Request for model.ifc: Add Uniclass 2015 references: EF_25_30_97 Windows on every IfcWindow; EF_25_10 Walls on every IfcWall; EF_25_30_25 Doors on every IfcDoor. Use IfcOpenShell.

First a look at what the model holds.

```python
import ifcopenshell

model = ifcopenshell.open("model.ifc")
print(model.schema)
print("classifications:", [c.Name for c in model.by_type("IfcClassification")])
for ifc_class in ("IfcDoor", "IfcRoof", "IfcStair", "IfcWall", "IfcWindow"):
    print(ifc_class, len(model.by_type(ifc_class)))
```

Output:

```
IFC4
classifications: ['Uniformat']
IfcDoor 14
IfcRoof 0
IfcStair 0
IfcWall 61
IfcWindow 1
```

```python
import ifcopenshell
import ifcopenshell.api.classification

model = ifcopenshell.open("model.ifc")

system = ifcopenshell.api.classification.add_classification(model, classification="Uniclass 2015")

codes = {
    "IfcWindow": ("EF_25_30_97", "Windows"),
    "IfcWall": ("EF_25_10", "Walls"),
    "IfcDoor": ("EF_25_30_25", "Doors"),
}
for ifc_class, (code, name) in codes.items():
    products = model.by_type(ifc_class)
    ifcopenshell.api.classification.add_reference(
        model, products=products, classification=system, identification=code, name=name
    )
    print(code, len(products))

model.write("model-out.ifc")
```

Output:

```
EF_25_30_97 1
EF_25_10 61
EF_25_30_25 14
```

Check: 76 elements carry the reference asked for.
